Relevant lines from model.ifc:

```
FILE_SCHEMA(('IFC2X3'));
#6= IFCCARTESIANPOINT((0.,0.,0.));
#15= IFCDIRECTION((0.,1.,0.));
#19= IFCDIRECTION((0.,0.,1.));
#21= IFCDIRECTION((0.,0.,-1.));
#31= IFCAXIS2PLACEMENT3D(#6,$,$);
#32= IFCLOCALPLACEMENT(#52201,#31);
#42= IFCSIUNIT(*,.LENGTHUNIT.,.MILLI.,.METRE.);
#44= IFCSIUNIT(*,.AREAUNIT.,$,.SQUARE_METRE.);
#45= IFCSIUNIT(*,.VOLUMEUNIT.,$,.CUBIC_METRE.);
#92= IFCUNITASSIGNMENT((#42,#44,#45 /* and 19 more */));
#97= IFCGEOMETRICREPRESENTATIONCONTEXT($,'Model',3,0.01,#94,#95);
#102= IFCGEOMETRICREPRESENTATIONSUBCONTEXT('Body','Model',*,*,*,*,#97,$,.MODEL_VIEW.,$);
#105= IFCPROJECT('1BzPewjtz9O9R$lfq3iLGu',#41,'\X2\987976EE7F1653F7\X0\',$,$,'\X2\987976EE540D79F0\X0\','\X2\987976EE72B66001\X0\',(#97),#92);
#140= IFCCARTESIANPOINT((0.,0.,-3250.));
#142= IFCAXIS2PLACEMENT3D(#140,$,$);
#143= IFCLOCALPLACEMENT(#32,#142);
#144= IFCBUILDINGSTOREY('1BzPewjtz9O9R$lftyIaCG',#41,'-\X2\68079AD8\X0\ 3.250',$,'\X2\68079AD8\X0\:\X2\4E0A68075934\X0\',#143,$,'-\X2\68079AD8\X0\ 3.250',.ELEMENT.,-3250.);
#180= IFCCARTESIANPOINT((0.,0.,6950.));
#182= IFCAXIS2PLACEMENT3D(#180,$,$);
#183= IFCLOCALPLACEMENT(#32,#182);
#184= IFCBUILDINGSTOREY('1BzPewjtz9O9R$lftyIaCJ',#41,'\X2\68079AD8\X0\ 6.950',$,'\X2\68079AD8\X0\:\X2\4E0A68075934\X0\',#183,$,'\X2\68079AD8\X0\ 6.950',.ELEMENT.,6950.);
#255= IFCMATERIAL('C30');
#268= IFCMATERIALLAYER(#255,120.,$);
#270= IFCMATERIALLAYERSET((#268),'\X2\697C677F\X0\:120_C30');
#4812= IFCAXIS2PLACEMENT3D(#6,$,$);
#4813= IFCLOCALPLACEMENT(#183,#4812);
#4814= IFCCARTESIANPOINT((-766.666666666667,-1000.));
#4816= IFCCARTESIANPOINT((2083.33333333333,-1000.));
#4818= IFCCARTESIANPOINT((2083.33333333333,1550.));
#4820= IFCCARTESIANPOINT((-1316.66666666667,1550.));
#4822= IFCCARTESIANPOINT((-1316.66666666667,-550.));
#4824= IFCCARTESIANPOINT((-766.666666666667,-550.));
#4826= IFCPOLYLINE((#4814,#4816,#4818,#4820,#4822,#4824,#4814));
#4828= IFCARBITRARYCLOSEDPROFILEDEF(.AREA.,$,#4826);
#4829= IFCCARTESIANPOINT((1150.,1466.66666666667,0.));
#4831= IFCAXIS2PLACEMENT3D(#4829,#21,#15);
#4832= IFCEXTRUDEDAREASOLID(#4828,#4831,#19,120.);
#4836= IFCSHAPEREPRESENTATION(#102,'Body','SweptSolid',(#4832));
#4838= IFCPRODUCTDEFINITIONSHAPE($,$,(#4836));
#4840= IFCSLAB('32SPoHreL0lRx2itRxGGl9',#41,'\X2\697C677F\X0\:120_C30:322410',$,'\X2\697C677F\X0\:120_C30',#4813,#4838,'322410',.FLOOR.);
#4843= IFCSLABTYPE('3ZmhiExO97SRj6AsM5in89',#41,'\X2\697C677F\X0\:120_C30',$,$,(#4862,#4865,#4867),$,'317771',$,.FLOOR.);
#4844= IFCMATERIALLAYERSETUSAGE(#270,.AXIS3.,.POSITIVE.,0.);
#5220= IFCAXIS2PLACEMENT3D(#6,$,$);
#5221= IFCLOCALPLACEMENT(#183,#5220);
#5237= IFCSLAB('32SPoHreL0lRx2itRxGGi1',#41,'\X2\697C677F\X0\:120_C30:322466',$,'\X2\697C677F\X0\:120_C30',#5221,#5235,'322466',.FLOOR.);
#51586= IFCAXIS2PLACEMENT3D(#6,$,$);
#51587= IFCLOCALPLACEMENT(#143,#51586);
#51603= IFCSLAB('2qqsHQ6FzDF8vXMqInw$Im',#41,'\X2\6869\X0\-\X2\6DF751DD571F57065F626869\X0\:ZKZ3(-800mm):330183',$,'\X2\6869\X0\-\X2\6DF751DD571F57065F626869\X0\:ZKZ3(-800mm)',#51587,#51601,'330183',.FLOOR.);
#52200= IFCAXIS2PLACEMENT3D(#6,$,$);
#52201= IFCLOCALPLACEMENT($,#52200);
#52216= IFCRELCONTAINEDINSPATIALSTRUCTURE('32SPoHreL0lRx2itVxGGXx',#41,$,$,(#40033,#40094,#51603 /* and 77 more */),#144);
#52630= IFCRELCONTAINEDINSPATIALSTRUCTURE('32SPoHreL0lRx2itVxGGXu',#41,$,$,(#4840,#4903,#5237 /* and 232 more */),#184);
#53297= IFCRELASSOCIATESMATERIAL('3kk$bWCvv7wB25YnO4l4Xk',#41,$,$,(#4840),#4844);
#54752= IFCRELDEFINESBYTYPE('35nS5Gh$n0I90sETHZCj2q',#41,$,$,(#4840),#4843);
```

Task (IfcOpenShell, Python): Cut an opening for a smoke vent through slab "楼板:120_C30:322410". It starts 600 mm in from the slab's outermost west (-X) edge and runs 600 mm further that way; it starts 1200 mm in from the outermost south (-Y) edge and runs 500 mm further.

```python
import numpy as np
import ifcopenshell
import ifcopenshell.api.feature
import ifcopenshell.api.geometry
import ifcopenshell.api.root
import ifcopenshell.geom
import ifcopenshell.util.placement
import ifcopenshell.util.representation
import ifcopenshell.util.shape
import ifcopenshell.util.unit

model = ifcopenshell.open("model.ifc")
unit_scale = ifcopenshell.util.unit.calculate_unit_scale(model)
settings = ifcopenshell.geom.settings()


def volume(element):
    """Net volume in cubic metres, openings subtracted."""
    shape = ifcopenshell.geom.create_shape(settings, element)
    return ifcopenshell.util.shape.get_volume(shape.geometry)


slab = model.by_guid("32SPoHreL0lRx2itRxGGl9")
before = volume(slab)

# Extent in the slab's own axes, in metres. The edges named are its -X and -Y sides.
slab_shape = ifcopenshell.geom.create_shape(settings, slab)
vertices = ifcopenshell.util.shape.get_vertices(slab_shape.geometry)
x_min, y_min, bottom = vertices.min(axis=0)
top = vertices[:, 2].max()

opening = ifcopenshell.api.root.create_entity(model, ifc_class="IfcOpeningElement", name="Smoke vent opening")
context = ifcopenshell.util.representation.get_context(model, "Model", "Body", "MODEL_VIEW")
width, depth = 0.6, 0.5
outline = [(0.0, 0.0), (width, 0.0), (width, depth), (0.0, depth), (0.0, 0.0)]
# Overshoot both faces by 50 mm so the cut is clean.
shape = ifcopenshell.api.geometry.add_slab_representation(
    model, context=context, depth=top - bottom + 0.1, polyline=outline
)
ifcopenshell.api.geometry.assign_representation(model, product=opening, representation=shape)

matrix = ifcopenshell.util.placement.get_local_placement(slab.ObjectPlacement)
matrix[:, 3] = matrix @ np.append(np.array([x_min + 0.6, y_min + 1.2, bottom - 0.05]) / unit_scale, 1.0)
ifcopenshell.api.geometry.edit_object_placement(model, product=opening, matrix=matrix, is_si=False)
ifcopenshell.api.feature.add_feature(model, feature=opening, element=slab)

after = volume(slab)

print(f"slab volume {before:.3f} -> {after:.3f} m3")

model.write("model_updated.ifc")
```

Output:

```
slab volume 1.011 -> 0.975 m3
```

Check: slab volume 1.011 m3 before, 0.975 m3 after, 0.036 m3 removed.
